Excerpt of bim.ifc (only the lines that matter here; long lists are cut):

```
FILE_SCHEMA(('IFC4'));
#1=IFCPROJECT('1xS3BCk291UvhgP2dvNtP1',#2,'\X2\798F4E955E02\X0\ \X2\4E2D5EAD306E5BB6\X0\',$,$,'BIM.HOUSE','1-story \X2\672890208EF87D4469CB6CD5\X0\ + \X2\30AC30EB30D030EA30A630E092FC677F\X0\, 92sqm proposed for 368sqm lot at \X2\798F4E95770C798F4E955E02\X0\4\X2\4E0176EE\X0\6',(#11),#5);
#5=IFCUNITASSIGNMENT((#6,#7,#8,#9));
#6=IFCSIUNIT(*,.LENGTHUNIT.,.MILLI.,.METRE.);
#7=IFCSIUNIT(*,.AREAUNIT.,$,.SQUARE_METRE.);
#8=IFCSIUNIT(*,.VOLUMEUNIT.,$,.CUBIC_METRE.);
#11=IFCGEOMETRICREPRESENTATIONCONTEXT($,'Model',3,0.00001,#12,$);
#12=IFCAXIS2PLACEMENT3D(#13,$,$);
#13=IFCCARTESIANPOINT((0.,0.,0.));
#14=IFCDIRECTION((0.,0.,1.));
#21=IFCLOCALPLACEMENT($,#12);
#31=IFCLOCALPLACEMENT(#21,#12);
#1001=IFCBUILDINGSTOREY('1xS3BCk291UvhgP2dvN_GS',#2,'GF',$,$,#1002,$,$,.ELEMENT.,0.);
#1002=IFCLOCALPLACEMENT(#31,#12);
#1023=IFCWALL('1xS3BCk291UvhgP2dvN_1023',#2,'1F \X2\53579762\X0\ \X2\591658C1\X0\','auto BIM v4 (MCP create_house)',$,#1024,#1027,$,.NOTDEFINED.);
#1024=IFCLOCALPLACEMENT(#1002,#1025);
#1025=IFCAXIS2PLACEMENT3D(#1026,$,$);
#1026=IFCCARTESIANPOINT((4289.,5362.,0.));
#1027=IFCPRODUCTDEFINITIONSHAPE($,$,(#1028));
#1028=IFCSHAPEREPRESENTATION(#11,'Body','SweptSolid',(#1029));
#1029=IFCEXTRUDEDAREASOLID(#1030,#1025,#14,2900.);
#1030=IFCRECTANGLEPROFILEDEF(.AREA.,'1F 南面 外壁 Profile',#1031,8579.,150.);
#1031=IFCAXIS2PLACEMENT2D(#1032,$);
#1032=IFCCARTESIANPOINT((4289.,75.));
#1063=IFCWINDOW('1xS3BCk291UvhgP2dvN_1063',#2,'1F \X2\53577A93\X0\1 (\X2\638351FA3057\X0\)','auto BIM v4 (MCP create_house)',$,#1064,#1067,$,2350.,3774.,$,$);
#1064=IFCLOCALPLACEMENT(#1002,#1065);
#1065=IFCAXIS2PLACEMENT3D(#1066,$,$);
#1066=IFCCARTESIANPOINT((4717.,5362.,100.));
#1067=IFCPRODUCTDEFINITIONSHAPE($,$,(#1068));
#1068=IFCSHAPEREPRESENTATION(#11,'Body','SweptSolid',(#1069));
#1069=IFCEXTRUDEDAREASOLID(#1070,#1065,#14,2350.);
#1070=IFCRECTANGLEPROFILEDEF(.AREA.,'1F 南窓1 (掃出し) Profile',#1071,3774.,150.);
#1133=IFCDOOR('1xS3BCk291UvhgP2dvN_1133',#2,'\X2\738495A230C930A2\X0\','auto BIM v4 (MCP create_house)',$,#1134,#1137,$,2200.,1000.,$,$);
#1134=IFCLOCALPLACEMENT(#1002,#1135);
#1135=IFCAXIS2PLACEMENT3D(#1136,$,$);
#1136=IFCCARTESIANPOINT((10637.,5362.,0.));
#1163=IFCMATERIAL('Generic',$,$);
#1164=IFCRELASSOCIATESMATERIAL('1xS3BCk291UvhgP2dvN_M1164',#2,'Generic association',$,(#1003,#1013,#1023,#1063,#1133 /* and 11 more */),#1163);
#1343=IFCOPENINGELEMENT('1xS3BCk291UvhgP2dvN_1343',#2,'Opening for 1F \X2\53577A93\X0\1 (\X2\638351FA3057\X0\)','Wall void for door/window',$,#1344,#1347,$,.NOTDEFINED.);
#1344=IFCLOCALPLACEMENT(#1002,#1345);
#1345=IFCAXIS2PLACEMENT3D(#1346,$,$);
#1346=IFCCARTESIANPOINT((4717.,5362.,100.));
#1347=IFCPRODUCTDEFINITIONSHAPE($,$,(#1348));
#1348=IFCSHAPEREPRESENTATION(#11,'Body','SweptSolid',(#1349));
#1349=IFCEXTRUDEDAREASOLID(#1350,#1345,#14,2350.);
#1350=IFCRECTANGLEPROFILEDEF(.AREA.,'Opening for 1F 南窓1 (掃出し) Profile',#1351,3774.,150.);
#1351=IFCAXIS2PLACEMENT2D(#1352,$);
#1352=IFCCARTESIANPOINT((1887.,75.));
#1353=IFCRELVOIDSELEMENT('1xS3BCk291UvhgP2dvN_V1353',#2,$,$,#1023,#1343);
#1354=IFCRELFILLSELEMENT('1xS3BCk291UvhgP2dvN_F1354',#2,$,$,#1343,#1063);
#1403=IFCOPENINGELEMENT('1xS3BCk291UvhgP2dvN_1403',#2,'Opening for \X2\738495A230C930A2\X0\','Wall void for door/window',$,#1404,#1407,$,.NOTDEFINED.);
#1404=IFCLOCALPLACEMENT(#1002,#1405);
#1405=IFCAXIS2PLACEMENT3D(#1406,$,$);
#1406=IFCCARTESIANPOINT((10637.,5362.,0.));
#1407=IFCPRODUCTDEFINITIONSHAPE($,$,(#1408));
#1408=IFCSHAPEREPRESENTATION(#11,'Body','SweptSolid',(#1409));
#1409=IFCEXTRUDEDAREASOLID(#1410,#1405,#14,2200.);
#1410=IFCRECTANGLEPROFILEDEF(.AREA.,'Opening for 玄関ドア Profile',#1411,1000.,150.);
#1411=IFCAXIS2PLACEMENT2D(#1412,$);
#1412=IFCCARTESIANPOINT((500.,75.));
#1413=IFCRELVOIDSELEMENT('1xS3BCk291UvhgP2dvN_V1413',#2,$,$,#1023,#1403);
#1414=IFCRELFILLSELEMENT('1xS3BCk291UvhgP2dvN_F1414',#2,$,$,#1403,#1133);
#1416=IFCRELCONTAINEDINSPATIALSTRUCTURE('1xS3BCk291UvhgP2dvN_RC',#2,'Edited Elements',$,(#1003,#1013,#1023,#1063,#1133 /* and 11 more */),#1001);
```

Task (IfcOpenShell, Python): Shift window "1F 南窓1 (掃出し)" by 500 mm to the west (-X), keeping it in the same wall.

```python
import ifcopenshell
import ifcopenshell.api.geometry
import ifcopenshell.util.placement
import ifcopenshell.util.unit

model = ifcopenshell.open("bim.ifc")
unit_scale = ifcopenshell.util.unit.calculate_unit_scale(model)

window = model.by_id(1063)
opening = window.FillsVoids[0].RelatingOpeningElement
wall = opening.VoidsElements[0].RelatingBuildingElement

wall_matrix = ifcopenshell.util.placement.get_local_placement(wall.ObjectPlacement)
shift = wall_matrix[:3, 0] * -0.5 / unit_scale
before = ifcopenshell.util.placement.get_local_placement(window.ObjectPlacement)[:3, 3].copy()

# The window is not placed relative to its opening, so move both.
for product in (opening, window):
    matrix = ifcopenshell.util.placement.get_local_placement(product.ObjectPlacement)
    matrix[:3, 3] += shift
    ifcopenshell.api.geometry.edit_object_placement(model, product=product, matrix=matrix, is_si=False)

after = ifcopenshell.util.placement.get_local_placement(window.ObjectPlacement)[:3, 3]
print("window moved by", (after - before).round(3) + 0.0)

model.write("bim_edited.ifc")
```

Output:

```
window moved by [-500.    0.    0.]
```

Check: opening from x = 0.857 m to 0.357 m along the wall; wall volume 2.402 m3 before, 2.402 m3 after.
